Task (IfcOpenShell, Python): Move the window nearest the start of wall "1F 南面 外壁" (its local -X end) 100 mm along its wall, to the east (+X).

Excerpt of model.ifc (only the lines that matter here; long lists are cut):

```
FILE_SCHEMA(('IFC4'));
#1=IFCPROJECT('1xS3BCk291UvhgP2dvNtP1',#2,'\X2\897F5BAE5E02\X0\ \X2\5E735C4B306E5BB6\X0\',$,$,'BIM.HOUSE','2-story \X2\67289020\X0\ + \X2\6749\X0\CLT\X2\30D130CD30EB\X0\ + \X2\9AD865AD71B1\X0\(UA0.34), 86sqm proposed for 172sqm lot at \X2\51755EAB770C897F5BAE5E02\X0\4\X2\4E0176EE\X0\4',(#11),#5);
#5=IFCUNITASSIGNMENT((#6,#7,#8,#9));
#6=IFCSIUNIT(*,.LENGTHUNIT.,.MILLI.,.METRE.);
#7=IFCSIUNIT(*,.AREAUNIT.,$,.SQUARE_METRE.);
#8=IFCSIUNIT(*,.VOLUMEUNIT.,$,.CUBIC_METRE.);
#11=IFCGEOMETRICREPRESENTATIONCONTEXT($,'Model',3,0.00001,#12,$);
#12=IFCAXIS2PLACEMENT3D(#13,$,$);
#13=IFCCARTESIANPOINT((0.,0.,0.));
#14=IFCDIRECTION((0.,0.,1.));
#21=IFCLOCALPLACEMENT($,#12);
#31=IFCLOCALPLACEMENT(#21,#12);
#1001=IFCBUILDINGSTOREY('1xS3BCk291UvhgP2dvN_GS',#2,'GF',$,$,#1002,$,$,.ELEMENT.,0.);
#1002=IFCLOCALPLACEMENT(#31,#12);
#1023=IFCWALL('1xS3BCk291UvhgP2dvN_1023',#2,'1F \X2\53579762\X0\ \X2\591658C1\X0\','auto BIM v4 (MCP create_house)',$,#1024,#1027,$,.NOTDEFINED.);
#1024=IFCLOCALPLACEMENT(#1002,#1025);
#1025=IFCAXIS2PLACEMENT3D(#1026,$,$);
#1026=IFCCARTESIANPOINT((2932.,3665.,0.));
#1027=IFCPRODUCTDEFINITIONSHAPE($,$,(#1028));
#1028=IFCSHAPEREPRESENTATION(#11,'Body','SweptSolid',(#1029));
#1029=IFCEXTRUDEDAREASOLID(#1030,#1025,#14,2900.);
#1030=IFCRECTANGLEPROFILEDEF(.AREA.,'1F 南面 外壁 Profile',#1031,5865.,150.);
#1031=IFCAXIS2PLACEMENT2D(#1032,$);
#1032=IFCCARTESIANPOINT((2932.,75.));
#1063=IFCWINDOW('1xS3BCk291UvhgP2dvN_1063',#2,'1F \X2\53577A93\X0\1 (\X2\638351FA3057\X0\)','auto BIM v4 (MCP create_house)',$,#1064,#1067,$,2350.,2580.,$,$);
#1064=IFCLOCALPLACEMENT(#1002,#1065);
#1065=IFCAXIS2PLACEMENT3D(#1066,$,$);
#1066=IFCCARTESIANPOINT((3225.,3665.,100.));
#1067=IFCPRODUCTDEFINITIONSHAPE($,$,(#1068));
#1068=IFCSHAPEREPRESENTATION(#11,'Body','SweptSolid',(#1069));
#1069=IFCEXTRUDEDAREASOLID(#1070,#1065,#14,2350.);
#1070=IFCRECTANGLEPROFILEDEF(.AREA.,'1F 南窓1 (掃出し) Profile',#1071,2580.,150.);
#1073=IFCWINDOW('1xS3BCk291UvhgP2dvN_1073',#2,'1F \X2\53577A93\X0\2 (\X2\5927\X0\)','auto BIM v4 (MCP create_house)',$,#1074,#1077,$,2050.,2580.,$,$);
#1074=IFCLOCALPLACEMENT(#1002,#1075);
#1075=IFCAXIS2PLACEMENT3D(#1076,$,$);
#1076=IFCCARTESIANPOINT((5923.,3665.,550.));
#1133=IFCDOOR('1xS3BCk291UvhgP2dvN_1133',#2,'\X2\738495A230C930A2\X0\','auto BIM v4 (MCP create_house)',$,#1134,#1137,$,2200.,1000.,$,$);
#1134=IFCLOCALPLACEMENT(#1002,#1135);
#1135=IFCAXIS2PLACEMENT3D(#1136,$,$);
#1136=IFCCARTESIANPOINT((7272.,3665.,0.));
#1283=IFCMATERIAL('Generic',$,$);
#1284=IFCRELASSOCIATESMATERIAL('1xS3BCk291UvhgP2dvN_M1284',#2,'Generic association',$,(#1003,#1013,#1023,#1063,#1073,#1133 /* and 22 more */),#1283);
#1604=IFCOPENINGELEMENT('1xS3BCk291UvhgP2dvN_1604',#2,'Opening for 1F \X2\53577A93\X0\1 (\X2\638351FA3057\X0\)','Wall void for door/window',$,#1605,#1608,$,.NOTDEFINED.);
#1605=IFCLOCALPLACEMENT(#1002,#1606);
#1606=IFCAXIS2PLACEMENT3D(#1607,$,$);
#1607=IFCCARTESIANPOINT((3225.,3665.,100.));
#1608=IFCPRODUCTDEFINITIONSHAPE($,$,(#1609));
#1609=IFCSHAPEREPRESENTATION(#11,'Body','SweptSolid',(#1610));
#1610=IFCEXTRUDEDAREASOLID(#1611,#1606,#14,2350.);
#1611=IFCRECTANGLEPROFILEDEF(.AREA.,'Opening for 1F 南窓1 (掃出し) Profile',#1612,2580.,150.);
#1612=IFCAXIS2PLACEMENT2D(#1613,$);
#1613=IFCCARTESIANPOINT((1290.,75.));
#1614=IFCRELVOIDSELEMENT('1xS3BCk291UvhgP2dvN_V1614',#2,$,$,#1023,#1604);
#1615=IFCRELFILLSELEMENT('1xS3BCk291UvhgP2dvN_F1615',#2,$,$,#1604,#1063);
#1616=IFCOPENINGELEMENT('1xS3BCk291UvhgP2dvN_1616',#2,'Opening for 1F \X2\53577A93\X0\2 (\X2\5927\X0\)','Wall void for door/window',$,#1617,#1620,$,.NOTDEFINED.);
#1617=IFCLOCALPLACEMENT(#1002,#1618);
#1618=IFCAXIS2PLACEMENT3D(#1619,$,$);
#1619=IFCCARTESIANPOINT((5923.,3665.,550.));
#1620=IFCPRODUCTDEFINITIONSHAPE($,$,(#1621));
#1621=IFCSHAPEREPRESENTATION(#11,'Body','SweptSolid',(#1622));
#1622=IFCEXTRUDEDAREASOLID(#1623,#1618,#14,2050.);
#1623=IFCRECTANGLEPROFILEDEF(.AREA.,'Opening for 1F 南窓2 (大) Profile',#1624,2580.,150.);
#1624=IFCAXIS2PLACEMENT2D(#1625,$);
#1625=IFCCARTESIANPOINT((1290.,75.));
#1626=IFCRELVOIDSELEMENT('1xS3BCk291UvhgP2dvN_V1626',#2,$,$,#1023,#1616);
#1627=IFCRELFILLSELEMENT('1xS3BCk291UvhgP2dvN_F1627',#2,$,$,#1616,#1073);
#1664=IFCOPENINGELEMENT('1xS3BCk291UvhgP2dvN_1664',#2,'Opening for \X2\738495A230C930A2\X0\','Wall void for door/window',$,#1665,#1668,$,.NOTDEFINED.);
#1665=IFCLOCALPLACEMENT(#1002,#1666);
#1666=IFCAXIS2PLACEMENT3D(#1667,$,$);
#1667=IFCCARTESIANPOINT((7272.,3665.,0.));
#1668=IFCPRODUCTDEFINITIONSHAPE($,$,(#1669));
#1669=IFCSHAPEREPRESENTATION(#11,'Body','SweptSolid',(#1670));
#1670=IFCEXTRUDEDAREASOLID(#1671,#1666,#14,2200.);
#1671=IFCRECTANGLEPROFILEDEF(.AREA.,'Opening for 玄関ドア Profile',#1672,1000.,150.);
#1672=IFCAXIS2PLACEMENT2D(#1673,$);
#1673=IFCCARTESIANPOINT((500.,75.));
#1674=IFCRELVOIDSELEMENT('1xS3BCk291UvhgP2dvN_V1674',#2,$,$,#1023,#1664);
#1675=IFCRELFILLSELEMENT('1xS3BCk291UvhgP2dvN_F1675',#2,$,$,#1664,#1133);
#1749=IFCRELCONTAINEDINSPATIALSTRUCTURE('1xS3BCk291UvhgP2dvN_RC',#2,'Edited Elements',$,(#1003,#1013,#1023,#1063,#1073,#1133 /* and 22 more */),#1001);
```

```python
import ifcopenshell
import ifcopenshell.api.geometry
import ifcopenshell.util.placement
import ifcopenshell.util.unit

model = ifcopenshell.open("model.ifc")
unit_scale = ifcopenshell.util.unit.calculate_unit_scale(model)

window = model.by_id(1063)
opening = window.FillsVoids[0].RelatingOpeningElement
wall = opening.VoidsElements[0].RelatingBuildingElement

wall_matrix = ifcopenshell.util.placement.get_local_placement(wall.ObjectPlacement)
shift = wall_matrix[:3, 0] * 0.1 / unit_scale
before = ifcopenshell.util.placement.get_local_placement(window.ObjectPlacement)[:3, 3].copy()

# The window is not placed relative to its opening, so move both.
for product in (opening, window):
    matrix = ifcopenshell.util.placement.get_local_placement(product.ObjectPlacement)
    matrix[:3, 3] += shift
    ifcopenshell.api.geometry.edit_object_placement(model, product=product, matrix=matrix, is_si=False)

after = ifcopenshell.util.placement.get_local_placement(window.ObjectPlacement)[:3, 3]
print("window moved by", (after - before).round(3) + 0.0)

model.write("model_edited.ifc")
```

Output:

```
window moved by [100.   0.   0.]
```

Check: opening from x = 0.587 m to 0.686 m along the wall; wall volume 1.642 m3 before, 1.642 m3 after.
